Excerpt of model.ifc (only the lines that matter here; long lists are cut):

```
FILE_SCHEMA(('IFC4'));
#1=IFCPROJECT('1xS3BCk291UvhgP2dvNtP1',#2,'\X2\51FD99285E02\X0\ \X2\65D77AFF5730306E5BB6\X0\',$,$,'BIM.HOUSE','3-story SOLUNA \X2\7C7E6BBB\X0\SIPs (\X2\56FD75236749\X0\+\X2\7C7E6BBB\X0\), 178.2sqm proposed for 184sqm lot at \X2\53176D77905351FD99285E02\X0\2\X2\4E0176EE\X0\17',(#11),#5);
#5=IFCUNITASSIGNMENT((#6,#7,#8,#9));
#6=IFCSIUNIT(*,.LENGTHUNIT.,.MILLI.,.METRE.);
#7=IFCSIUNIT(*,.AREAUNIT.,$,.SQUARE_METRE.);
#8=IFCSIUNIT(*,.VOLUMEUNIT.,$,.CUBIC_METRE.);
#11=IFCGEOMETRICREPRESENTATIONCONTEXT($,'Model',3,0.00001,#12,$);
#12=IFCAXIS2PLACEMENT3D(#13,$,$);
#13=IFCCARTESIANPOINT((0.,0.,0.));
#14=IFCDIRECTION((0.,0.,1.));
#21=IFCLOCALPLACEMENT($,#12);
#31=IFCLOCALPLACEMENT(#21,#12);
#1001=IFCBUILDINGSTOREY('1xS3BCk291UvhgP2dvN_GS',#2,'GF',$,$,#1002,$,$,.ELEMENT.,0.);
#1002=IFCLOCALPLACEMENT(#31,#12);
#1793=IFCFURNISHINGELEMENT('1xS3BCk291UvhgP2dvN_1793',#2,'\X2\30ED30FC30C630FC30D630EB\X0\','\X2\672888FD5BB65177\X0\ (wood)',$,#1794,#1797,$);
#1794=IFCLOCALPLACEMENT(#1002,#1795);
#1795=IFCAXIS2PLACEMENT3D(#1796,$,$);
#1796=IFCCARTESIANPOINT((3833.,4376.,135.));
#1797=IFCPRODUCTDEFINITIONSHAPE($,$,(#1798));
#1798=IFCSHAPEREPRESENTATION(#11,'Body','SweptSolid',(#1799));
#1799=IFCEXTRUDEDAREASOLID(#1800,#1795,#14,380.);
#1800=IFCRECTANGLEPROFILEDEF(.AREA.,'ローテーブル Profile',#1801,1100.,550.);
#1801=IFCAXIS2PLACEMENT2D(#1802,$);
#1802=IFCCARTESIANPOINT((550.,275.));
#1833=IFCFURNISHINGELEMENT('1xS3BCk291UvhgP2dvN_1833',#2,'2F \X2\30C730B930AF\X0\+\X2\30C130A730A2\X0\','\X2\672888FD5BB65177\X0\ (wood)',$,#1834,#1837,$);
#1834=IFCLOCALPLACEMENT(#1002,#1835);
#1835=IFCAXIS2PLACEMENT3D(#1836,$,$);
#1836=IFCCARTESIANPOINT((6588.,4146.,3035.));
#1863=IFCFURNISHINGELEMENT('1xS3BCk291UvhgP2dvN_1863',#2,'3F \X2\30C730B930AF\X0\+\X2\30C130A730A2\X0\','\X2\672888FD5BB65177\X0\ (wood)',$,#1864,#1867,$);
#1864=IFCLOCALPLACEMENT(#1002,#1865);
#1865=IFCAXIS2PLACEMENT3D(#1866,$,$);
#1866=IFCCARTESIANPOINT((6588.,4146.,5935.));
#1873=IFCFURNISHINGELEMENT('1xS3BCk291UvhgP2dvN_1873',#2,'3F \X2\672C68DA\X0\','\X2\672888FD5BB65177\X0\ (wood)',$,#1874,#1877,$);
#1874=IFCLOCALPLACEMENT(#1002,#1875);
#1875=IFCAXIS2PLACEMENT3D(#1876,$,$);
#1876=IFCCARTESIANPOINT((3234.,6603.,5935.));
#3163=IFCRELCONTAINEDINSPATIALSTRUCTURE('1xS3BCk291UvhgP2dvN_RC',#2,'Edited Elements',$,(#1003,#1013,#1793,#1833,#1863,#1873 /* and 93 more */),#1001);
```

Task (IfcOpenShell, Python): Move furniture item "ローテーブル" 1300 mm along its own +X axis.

```python
import ifcopenshell
import ifcopenshell.api.geometry
import ifcopenshell.util.placement
import ifcopenshell.util.unit

model = ifcopenshell.open("model.ifc")
unit_scale = ifcopenshell.util.unit.calculate_unit_scale(model)

item = model.by_id(1793)
matrix = ifcopenshell.util.placement.get_local_placement(item.ObjectPlacement)
matrix[:3, 3] += matrix[:3, 0] * 1.3 / unit_scale
ifcopenshell.api.geometry.edit_object_placement(model, product=item, matrix=matrix, is_si=False)

print(ifcopenshell.util.placement.get_local_placement(item.ObjectPlacement).round(3) + 0.0)

model.write("model_edited.ifc")
```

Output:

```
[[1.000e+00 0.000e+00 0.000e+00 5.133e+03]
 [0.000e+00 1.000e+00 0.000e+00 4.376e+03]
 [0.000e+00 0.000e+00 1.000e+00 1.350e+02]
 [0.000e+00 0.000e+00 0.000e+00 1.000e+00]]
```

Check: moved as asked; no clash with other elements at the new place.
